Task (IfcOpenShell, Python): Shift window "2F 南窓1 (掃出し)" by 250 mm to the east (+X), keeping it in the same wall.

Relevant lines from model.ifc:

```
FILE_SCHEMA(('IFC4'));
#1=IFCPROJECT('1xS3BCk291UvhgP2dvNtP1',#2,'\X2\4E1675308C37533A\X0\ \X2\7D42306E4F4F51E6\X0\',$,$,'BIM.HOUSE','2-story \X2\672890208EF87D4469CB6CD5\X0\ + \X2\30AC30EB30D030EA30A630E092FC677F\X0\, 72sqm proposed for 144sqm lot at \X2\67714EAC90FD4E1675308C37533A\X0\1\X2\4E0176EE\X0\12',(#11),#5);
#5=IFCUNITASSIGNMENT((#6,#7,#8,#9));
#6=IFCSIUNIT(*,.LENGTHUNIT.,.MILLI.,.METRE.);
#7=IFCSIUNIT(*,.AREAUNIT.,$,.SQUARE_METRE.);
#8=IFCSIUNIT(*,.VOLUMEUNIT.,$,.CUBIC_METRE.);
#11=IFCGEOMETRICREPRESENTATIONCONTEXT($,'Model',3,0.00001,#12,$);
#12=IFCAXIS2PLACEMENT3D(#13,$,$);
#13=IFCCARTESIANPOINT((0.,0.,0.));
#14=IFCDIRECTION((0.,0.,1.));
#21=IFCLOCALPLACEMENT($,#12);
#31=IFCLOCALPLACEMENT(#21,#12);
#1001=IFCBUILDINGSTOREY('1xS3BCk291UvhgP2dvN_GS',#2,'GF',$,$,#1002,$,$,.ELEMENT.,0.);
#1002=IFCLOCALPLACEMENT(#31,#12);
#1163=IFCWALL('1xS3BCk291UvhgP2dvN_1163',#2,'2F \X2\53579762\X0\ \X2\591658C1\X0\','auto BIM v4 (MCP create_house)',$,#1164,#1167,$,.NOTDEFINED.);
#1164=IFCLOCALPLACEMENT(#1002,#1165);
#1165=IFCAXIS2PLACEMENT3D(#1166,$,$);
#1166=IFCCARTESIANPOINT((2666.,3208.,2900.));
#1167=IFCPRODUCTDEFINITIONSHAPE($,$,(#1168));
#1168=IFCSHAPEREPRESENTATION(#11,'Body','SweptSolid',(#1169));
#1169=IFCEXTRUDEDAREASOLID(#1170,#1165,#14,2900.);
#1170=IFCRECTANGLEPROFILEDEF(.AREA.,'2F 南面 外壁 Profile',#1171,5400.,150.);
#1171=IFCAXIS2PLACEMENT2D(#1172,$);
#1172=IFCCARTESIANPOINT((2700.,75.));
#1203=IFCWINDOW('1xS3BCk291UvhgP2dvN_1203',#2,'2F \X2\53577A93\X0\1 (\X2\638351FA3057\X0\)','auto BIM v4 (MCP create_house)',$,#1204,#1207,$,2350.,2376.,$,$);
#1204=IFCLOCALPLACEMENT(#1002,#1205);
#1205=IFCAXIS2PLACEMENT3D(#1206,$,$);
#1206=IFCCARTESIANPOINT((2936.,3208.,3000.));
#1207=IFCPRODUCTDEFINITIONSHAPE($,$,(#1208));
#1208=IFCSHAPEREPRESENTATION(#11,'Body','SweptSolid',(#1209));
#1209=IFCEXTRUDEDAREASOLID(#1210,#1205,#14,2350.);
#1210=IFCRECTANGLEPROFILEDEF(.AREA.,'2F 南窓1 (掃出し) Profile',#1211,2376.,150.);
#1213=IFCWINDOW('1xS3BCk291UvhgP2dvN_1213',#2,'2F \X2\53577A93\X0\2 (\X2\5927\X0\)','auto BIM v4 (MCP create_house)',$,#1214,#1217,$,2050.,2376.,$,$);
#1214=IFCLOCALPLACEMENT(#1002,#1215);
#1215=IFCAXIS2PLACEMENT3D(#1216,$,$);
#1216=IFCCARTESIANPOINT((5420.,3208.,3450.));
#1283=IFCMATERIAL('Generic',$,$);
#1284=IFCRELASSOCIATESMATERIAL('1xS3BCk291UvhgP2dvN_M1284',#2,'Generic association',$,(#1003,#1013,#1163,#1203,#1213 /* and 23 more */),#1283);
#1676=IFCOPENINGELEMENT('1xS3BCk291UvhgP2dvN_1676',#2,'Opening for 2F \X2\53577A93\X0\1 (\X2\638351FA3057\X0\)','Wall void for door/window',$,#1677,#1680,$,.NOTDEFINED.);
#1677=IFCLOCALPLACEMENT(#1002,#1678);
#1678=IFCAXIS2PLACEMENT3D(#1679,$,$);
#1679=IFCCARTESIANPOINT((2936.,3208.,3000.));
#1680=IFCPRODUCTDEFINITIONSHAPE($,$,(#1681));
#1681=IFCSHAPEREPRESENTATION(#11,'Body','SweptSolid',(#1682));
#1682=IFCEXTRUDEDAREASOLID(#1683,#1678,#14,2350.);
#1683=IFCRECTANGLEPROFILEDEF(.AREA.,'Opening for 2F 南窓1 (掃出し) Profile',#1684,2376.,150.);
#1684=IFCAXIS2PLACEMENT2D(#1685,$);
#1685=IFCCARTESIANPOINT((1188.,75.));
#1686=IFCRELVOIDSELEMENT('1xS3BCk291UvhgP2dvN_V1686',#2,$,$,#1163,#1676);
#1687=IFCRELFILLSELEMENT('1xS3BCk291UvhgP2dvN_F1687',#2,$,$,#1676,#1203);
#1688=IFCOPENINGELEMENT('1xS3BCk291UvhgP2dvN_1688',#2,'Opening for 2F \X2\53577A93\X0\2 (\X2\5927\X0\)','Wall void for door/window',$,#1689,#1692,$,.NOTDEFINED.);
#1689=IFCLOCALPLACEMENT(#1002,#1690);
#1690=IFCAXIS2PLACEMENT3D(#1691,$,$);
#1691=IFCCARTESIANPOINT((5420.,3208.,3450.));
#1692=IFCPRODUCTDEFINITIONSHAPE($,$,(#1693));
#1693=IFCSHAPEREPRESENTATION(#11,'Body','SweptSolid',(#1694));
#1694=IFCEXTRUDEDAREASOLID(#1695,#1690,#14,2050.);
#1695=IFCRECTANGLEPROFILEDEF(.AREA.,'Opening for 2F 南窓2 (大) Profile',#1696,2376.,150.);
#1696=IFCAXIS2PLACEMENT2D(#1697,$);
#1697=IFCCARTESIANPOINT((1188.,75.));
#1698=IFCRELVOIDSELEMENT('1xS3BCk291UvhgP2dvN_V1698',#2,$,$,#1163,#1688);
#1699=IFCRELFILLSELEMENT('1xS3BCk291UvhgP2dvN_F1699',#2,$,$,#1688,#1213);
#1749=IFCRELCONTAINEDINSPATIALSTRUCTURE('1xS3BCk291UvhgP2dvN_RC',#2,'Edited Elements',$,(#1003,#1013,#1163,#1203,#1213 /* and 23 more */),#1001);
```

```python
import ifcopenshell
import ifcopenshell.api.geometry
import ifcopenshell.util.placement

model = ifcopenshell.open("model.ifc")

window = model.by_guid("1xS3BCk291UvhgP2dvN_1203")
opening = window.FillsVoids[0].RelatingOpeningElement
wall = opening.VoidsElements[0].RelatingBuildingElement

wall_matrix = ifcopenshell.util.placement.get_local_placement(wall.ObjectPlacement)
shift = wall_matrix[:3, 0] * 250.0
before = ifcopenshell.util.placement.get_local_placement(window.ObjectPlacement)[:3, 3].copy()

# The window is not placed relative to its opening, so move both.
for product in (opening, window):
    matrix = ifcopenshell.util.placement.get_local_placement(product.ObjectPlacement)
    matrix[:3, 3] += shift
    ifcopenshell.api.geometry.edit_object_placement(model, product=product, matrix=matrix, is_si=False)

after = ifcopenshell.util.placement.get_local_placement(window.ObjectPlacement)[:3, 3]
print("window moved by", (after - before).round(3) + 0.0)

model.write("model_updated.ifc")
```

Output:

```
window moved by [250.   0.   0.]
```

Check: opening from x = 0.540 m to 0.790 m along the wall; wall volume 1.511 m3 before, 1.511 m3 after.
